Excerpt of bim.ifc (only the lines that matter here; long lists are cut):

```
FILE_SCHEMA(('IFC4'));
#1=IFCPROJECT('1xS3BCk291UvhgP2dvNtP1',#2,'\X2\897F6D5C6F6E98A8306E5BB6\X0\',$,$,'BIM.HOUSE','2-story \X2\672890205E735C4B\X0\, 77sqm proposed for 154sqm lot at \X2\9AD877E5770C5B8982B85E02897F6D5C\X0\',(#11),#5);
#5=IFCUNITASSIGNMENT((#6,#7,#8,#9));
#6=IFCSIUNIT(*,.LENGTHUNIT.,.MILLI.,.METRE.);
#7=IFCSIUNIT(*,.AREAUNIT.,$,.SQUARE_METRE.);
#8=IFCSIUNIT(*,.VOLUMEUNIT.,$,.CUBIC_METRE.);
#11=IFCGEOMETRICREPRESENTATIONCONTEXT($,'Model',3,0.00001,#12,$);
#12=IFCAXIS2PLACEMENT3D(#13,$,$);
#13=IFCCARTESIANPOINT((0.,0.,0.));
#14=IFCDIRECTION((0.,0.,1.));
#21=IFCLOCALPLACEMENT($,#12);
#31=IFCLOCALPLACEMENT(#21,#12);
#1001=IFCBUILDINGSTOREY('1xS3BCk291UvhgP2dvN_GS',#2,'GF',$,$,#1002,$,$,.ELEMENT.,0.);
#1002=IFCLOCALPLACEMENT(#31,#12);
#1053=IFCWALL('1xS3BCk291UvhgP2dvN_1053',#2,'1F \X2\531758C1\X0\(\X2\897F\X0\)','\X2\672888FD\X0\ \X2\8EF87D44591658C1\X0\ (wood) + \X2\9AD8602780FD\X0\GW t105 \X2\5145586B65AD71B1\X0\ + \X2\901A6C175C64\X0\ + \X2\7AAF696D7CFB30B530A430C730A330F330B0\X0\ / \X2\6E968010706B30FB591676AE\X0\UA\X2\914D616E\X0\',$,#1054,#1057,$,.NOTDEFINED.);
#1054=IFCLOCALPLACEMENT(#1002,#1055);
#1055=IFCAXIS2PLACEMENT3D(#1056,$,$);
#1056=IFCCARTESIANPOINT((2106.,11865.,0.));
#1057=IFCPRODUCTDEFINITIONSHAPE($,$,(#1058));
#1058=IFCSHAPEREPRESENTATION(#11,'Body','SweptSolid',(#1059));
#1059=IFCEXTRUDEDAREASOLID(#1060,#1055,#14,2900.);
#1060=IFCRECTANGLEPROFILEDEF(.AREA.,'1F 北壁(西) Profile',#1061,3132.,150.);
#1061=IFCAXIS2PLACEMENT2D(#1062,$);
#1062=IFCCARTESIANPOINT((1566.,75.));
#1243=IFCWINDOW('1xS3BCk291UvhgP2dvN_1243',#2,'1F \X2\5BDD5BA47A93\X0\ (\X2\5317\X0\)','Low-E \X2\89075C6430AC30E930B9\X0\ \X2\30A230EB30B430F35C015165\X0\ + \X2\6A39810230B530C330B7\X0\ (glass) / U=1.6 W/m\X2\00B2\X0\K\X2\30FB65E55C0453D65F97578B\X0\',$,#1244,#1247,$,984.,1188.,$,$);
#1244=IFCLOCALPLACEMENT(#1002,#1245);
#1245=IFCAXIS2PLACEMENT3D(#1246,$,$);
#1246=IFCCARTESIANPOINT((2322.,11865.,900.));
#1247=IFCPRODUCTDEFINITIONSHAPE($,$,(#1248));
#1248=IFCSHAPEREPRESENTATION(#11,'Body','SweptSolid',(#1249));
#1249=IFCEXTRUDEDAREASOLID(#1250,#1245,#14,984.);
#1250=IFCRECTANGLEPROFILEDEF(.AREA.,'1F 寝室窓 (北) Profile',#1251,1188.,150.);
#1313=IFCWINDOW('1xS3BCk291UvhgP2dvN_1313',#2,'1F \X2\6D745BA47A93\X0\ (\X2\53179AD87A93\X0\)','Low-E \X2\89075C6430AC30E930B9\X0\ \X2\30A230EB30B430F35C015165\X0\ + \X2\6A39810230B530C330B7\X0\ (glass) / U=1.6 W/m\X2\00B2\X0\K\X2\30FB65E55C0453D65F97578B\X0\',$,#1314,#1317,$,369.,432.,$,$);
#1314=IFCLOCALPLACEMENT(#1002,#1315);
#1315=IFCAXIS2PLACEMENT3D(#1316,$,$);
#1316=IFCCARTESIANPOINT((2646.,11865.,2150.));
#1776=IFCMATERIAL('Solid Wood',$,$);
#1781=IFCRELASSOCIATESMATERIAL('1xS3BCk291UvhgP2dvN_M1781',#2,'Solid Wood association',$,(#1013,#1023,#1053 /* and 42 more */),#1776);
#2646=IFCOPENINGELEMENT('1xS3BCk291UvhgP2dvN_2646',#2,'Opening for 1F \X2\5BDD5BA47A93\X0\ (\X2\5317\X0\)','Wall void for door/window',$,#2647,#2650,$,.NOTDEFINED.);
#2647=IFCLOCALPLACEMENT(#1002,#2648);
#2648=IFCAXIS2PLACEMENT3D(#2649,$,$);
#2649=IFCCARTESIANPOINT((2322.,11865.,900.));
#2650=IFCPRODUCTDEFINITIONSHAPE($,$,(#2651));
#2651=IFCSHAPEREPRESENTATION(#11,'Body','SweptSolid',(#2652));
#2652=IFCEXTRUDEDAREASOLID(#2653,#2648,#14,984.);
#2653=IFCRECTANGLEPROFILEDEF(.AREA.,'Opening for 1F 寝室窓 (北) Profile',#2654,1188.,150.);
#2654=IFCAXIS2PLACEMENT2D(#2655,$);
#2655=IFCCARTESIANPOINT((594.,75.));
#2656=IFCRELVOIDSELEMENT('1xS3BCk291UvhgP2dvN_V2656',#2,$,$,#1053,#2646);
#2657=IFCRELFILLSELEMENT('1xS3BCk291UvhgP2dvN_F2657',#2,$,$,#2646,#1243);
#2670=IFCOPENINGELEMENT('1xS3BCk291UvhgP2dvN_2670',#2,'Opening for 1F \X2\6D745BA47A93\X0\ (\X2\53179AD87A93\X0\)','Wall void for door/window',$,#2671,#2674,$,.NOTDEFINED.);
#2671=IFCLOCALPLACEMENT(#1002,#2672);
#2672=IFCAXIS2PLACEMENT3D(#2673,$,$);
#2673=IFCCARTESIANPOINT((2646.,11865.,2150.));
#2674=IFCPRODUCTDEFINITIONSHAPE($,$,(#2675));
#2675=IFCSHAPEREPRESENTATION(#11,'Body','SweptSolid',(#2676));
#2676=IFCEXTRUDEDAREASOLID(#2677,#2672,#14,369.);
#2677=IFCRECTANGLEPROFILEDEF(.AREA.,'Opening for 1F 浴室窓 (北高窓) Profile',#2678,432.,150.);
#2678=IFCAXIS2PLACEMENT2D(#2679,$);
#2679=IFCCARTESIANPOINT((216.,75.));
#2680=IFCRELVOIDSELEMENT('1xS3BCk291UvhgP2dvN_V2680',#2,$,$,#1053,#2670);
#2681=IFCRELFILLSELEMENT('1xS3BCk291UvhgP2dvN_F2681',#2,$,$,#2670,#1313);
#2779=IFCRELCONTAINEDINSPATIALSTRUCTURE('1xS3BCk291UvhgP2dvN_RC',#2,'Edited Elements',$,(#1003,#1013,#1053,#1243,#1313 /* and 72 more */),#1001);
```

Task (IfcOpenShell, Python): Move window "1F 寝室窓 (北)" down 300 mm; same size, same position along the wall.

```python
import numpy as np
import ifcopenshell
import ifcopenshell.api.geometry
import ifcopenshell.util.placement
import ifcopenshell.util.unit

model = ifcopenshell.open("bim.ifc")
unit_scale = ifcopenshell.util.unit.calculate_unit_scale(model)

window = model.by_id(1243)
opening = window.FillsVoids[0].RelatingOpeningElement
dz = -0.3 / unit_scale

shift = np.array([0.0, 0.0, dz])
# The window is not placed relative to its opening, so move both.
for product in (opening, window):
    matrix = ifcopenshell.util.placement.get_local_placement(product.ObjectPlacement)
    matrix[:3, 3] += shift
    ifcopenshell.api.geometry.edit_object_placement(model, product=product, matrix=matrix, is_si=False)

print(f"moved by {dz * unit_scale:+.3f} m")

model.write("bim_edited.ifc")
```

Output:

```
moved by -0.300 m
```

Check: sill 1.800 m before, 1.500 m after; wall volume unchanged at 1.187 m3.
